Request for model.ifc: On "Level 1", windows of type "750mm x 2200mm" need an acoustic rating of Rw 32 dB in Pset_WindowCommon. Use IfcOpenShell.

First a look at what the model holds.

```python
import ifcopenshell
import ifcopenshell.util.element

model = ifcopenshell.open("model.ifc")
print(model.schema)
storey = next(s for s in model.by_type("IfcBuildingStorey") if s.Name == "Level 1")
windows = [e for e in ifcopenshell.util.element.get_decomposition(storey) if e.is_a("IfcWindow")]
seen = {}
for e in windows:
    element_type = ifcopenshell.util.element.get_type(e)
    key = (element_type.Name if element_type != e and element_type else None, ifcopenshell.util.element.get_pset(e, "Pset_WindowCommon", "AcousticRating"))
    seen[key] = seen.get(key, 0) + 1
for (name, value), count in sorted(seen.items(), key=str):
    print(count, "x", name, "|", value)
```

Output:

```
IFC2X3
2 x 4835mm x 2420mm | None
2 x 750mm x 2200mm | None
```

```python
import ifcopenshell
import ifcopenshell.api.pset
import ifcopenshell.util.element

model = ifcopenshell.open("model.ifc")

storey = next(s for s in model.by_type("IfcBuildingStorey") if s.Name == "Level 1")
windows = [e for e in ifcopenshell.util.element.get_decomposition(storey) if e.is_a("IfcWindow")]

count = 0
for e in windows:
    element_type = ifcopenshell.util.element.get_type(e)
    if element_type in (None, e) or element_type.Name != "750mm x 2200mm":
        continue
    # add_pset returns the element's existing set when there is one.
    pset = ifcopenshell.api.pset.add_pset(model, product=e, name="Pset_WindowCommon")
    ifcopenshell.api.pset.edit_pset(model, pset=pset, properties={"AcousticRating": "Rw 32 dB"})
    count += 1

print(count, "windows updated")

model.write("model_v2.ifc")
```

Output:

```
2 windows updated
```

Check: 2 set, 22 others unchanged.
